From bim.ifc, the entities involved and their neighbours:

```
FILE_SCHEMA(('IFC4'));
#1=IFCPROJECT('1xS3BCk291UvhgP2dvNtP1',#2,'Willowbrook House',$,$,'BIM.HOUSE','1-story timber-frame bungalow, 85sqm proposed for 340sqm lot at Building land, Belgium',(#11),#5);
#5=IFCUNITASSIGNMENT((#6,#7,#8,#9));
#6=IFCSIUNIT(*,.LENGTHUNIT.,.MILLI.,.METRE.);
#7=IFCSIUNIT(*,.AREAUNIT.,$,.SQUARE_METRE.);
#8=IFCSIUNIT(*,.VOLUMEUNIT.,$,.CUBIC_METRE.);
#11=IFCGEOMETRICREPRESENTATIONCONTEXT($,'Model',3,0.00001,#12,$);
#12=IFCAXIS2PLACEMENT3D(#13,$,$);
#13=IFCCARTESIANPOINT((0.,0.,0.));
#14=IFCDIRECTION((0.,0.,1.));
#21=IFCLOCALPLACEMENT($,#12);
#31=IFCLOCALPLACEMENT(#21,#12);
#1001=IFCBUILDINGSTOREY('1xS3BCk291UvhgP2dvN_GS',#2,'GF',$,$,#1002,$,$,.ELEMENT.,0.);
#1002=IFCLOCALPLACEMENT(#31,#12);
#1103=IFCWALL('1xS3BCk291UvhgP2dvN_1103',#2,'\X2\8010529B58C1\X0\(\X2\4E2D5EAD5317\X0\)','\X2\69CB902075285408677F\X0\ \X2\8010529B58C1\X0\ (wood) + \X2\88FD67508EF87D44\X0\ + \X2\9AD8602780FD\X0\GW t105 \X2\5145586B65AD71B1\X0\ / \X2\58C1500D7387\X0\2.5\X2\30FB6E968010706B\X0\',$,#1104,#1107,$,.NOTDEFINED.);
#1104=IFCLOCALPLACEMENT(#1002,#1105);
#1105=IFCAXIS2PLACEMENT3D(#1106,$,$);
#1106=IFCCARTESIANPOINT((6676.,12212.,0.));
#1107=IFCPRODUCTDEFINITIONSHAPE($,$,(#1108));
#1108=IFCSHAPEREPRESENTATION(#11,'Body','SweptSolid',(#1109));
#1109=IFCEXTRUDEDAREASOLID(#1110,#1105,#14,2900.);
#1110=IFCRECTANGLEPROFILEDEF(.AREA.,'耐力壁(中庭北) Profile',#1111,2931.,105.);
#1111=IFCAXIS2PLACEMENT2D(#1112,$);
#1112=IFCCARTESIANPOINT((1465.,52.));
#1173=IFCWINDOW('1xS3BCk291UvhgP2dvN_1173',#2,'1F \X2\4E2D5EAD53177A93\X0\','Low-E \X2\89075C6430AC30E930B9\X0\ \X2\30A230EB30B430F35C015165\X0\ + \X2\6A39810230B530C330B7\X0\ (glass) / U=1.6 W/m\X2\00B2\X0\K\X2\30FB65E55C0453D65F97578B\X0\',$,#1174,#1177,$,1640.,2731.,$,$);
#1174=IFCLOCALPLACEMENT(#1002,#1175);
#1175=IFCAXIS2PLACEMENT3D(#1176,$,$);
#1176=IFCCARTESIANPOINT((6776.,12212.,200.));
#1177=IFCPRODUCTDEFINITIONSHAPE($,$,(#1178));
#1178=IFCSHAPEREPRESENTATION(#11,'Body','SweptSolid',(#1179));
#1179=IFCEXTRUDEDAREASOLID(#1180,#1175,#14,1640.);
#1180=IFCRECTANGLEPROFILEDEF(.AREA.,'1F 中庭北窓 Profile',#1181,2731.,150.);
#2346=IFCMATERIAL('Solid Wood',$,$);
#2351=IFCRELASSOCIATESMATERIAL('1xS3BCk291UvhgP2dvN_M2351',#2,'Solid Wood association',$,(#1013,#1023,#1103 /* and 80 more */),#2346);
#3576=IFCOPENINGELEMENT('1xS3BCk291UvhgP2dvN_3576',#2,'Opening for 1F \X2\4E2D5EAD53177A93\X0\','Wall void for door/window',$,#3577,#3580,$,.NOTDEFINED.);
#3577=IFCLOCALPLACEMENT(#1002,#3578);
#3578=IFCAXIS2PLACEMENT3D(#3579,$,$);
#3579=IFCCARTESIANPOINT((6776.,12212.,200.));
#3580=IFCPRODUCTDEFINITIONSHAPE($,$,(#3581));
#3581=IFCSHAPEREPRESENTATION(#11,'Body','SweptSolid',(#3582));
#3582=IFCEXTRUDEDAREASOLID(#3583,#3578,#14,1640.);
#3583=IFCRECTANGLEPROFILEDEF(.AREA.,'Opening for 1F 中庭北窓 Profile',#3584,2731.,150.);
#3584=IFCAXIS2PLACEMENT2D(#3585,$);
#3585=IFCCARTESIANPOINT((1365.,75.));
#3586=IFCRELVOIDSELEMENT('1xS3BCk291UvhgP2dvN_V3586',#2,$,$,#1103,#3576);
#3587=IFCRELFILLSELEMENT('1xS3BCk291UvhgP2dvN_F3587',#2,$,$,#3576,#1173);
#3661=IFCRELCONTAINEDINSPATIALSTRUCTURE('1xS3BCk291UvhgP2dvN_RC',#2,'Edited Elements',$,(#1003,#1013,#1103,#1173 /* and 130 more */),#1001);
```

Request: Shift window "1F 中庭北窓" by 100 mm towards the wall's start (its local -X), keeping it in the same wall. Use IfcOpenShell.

```python
import ifcopenshell
import ifcopenshell.api.geometry
import ifcopenshell.util.placement

model = ifcopenshell.open("bim.ifc")

window = model.by_guid("1xS3BCk291UvhgP2dvN_1173")
opening = window.FillsVoids[0].RelatingOpeningElement
wall = opening.VoidsElements[0].RelatingBuildingElement

wall_matrix = ifcopenshell.util.placement.get_local_placement(wall.ObjectPlacement)
shift = wall_matrix[:3, 0] * -100.0
before = ifcopenshell.util.placement.get_local_placement(window.ObjectPlacement)[:3, 3].copy()

# The window is not placed relative to its opening, so move both.
for product in (opening, window):
    matrix = ifcopenshell.util.placement.get_local_placement(product.ObjectPlacement)
    matrix[:3, 3] += shift
    ifcopenshell.api.geometry.edit_object_placement(model, product=product, matrix=matrix, is_si=False)

after = ifcopenshell.util.placement.get_local_placement(window.ObjectPlacement)[:3, 3]
print("window moved by", (after - before).round(3) + 0.0)

model.write("bim_edited.ifc")
```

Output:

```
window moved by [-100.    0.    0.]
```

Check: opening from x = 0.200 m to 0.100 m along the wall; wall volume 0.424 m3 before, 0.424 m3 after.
